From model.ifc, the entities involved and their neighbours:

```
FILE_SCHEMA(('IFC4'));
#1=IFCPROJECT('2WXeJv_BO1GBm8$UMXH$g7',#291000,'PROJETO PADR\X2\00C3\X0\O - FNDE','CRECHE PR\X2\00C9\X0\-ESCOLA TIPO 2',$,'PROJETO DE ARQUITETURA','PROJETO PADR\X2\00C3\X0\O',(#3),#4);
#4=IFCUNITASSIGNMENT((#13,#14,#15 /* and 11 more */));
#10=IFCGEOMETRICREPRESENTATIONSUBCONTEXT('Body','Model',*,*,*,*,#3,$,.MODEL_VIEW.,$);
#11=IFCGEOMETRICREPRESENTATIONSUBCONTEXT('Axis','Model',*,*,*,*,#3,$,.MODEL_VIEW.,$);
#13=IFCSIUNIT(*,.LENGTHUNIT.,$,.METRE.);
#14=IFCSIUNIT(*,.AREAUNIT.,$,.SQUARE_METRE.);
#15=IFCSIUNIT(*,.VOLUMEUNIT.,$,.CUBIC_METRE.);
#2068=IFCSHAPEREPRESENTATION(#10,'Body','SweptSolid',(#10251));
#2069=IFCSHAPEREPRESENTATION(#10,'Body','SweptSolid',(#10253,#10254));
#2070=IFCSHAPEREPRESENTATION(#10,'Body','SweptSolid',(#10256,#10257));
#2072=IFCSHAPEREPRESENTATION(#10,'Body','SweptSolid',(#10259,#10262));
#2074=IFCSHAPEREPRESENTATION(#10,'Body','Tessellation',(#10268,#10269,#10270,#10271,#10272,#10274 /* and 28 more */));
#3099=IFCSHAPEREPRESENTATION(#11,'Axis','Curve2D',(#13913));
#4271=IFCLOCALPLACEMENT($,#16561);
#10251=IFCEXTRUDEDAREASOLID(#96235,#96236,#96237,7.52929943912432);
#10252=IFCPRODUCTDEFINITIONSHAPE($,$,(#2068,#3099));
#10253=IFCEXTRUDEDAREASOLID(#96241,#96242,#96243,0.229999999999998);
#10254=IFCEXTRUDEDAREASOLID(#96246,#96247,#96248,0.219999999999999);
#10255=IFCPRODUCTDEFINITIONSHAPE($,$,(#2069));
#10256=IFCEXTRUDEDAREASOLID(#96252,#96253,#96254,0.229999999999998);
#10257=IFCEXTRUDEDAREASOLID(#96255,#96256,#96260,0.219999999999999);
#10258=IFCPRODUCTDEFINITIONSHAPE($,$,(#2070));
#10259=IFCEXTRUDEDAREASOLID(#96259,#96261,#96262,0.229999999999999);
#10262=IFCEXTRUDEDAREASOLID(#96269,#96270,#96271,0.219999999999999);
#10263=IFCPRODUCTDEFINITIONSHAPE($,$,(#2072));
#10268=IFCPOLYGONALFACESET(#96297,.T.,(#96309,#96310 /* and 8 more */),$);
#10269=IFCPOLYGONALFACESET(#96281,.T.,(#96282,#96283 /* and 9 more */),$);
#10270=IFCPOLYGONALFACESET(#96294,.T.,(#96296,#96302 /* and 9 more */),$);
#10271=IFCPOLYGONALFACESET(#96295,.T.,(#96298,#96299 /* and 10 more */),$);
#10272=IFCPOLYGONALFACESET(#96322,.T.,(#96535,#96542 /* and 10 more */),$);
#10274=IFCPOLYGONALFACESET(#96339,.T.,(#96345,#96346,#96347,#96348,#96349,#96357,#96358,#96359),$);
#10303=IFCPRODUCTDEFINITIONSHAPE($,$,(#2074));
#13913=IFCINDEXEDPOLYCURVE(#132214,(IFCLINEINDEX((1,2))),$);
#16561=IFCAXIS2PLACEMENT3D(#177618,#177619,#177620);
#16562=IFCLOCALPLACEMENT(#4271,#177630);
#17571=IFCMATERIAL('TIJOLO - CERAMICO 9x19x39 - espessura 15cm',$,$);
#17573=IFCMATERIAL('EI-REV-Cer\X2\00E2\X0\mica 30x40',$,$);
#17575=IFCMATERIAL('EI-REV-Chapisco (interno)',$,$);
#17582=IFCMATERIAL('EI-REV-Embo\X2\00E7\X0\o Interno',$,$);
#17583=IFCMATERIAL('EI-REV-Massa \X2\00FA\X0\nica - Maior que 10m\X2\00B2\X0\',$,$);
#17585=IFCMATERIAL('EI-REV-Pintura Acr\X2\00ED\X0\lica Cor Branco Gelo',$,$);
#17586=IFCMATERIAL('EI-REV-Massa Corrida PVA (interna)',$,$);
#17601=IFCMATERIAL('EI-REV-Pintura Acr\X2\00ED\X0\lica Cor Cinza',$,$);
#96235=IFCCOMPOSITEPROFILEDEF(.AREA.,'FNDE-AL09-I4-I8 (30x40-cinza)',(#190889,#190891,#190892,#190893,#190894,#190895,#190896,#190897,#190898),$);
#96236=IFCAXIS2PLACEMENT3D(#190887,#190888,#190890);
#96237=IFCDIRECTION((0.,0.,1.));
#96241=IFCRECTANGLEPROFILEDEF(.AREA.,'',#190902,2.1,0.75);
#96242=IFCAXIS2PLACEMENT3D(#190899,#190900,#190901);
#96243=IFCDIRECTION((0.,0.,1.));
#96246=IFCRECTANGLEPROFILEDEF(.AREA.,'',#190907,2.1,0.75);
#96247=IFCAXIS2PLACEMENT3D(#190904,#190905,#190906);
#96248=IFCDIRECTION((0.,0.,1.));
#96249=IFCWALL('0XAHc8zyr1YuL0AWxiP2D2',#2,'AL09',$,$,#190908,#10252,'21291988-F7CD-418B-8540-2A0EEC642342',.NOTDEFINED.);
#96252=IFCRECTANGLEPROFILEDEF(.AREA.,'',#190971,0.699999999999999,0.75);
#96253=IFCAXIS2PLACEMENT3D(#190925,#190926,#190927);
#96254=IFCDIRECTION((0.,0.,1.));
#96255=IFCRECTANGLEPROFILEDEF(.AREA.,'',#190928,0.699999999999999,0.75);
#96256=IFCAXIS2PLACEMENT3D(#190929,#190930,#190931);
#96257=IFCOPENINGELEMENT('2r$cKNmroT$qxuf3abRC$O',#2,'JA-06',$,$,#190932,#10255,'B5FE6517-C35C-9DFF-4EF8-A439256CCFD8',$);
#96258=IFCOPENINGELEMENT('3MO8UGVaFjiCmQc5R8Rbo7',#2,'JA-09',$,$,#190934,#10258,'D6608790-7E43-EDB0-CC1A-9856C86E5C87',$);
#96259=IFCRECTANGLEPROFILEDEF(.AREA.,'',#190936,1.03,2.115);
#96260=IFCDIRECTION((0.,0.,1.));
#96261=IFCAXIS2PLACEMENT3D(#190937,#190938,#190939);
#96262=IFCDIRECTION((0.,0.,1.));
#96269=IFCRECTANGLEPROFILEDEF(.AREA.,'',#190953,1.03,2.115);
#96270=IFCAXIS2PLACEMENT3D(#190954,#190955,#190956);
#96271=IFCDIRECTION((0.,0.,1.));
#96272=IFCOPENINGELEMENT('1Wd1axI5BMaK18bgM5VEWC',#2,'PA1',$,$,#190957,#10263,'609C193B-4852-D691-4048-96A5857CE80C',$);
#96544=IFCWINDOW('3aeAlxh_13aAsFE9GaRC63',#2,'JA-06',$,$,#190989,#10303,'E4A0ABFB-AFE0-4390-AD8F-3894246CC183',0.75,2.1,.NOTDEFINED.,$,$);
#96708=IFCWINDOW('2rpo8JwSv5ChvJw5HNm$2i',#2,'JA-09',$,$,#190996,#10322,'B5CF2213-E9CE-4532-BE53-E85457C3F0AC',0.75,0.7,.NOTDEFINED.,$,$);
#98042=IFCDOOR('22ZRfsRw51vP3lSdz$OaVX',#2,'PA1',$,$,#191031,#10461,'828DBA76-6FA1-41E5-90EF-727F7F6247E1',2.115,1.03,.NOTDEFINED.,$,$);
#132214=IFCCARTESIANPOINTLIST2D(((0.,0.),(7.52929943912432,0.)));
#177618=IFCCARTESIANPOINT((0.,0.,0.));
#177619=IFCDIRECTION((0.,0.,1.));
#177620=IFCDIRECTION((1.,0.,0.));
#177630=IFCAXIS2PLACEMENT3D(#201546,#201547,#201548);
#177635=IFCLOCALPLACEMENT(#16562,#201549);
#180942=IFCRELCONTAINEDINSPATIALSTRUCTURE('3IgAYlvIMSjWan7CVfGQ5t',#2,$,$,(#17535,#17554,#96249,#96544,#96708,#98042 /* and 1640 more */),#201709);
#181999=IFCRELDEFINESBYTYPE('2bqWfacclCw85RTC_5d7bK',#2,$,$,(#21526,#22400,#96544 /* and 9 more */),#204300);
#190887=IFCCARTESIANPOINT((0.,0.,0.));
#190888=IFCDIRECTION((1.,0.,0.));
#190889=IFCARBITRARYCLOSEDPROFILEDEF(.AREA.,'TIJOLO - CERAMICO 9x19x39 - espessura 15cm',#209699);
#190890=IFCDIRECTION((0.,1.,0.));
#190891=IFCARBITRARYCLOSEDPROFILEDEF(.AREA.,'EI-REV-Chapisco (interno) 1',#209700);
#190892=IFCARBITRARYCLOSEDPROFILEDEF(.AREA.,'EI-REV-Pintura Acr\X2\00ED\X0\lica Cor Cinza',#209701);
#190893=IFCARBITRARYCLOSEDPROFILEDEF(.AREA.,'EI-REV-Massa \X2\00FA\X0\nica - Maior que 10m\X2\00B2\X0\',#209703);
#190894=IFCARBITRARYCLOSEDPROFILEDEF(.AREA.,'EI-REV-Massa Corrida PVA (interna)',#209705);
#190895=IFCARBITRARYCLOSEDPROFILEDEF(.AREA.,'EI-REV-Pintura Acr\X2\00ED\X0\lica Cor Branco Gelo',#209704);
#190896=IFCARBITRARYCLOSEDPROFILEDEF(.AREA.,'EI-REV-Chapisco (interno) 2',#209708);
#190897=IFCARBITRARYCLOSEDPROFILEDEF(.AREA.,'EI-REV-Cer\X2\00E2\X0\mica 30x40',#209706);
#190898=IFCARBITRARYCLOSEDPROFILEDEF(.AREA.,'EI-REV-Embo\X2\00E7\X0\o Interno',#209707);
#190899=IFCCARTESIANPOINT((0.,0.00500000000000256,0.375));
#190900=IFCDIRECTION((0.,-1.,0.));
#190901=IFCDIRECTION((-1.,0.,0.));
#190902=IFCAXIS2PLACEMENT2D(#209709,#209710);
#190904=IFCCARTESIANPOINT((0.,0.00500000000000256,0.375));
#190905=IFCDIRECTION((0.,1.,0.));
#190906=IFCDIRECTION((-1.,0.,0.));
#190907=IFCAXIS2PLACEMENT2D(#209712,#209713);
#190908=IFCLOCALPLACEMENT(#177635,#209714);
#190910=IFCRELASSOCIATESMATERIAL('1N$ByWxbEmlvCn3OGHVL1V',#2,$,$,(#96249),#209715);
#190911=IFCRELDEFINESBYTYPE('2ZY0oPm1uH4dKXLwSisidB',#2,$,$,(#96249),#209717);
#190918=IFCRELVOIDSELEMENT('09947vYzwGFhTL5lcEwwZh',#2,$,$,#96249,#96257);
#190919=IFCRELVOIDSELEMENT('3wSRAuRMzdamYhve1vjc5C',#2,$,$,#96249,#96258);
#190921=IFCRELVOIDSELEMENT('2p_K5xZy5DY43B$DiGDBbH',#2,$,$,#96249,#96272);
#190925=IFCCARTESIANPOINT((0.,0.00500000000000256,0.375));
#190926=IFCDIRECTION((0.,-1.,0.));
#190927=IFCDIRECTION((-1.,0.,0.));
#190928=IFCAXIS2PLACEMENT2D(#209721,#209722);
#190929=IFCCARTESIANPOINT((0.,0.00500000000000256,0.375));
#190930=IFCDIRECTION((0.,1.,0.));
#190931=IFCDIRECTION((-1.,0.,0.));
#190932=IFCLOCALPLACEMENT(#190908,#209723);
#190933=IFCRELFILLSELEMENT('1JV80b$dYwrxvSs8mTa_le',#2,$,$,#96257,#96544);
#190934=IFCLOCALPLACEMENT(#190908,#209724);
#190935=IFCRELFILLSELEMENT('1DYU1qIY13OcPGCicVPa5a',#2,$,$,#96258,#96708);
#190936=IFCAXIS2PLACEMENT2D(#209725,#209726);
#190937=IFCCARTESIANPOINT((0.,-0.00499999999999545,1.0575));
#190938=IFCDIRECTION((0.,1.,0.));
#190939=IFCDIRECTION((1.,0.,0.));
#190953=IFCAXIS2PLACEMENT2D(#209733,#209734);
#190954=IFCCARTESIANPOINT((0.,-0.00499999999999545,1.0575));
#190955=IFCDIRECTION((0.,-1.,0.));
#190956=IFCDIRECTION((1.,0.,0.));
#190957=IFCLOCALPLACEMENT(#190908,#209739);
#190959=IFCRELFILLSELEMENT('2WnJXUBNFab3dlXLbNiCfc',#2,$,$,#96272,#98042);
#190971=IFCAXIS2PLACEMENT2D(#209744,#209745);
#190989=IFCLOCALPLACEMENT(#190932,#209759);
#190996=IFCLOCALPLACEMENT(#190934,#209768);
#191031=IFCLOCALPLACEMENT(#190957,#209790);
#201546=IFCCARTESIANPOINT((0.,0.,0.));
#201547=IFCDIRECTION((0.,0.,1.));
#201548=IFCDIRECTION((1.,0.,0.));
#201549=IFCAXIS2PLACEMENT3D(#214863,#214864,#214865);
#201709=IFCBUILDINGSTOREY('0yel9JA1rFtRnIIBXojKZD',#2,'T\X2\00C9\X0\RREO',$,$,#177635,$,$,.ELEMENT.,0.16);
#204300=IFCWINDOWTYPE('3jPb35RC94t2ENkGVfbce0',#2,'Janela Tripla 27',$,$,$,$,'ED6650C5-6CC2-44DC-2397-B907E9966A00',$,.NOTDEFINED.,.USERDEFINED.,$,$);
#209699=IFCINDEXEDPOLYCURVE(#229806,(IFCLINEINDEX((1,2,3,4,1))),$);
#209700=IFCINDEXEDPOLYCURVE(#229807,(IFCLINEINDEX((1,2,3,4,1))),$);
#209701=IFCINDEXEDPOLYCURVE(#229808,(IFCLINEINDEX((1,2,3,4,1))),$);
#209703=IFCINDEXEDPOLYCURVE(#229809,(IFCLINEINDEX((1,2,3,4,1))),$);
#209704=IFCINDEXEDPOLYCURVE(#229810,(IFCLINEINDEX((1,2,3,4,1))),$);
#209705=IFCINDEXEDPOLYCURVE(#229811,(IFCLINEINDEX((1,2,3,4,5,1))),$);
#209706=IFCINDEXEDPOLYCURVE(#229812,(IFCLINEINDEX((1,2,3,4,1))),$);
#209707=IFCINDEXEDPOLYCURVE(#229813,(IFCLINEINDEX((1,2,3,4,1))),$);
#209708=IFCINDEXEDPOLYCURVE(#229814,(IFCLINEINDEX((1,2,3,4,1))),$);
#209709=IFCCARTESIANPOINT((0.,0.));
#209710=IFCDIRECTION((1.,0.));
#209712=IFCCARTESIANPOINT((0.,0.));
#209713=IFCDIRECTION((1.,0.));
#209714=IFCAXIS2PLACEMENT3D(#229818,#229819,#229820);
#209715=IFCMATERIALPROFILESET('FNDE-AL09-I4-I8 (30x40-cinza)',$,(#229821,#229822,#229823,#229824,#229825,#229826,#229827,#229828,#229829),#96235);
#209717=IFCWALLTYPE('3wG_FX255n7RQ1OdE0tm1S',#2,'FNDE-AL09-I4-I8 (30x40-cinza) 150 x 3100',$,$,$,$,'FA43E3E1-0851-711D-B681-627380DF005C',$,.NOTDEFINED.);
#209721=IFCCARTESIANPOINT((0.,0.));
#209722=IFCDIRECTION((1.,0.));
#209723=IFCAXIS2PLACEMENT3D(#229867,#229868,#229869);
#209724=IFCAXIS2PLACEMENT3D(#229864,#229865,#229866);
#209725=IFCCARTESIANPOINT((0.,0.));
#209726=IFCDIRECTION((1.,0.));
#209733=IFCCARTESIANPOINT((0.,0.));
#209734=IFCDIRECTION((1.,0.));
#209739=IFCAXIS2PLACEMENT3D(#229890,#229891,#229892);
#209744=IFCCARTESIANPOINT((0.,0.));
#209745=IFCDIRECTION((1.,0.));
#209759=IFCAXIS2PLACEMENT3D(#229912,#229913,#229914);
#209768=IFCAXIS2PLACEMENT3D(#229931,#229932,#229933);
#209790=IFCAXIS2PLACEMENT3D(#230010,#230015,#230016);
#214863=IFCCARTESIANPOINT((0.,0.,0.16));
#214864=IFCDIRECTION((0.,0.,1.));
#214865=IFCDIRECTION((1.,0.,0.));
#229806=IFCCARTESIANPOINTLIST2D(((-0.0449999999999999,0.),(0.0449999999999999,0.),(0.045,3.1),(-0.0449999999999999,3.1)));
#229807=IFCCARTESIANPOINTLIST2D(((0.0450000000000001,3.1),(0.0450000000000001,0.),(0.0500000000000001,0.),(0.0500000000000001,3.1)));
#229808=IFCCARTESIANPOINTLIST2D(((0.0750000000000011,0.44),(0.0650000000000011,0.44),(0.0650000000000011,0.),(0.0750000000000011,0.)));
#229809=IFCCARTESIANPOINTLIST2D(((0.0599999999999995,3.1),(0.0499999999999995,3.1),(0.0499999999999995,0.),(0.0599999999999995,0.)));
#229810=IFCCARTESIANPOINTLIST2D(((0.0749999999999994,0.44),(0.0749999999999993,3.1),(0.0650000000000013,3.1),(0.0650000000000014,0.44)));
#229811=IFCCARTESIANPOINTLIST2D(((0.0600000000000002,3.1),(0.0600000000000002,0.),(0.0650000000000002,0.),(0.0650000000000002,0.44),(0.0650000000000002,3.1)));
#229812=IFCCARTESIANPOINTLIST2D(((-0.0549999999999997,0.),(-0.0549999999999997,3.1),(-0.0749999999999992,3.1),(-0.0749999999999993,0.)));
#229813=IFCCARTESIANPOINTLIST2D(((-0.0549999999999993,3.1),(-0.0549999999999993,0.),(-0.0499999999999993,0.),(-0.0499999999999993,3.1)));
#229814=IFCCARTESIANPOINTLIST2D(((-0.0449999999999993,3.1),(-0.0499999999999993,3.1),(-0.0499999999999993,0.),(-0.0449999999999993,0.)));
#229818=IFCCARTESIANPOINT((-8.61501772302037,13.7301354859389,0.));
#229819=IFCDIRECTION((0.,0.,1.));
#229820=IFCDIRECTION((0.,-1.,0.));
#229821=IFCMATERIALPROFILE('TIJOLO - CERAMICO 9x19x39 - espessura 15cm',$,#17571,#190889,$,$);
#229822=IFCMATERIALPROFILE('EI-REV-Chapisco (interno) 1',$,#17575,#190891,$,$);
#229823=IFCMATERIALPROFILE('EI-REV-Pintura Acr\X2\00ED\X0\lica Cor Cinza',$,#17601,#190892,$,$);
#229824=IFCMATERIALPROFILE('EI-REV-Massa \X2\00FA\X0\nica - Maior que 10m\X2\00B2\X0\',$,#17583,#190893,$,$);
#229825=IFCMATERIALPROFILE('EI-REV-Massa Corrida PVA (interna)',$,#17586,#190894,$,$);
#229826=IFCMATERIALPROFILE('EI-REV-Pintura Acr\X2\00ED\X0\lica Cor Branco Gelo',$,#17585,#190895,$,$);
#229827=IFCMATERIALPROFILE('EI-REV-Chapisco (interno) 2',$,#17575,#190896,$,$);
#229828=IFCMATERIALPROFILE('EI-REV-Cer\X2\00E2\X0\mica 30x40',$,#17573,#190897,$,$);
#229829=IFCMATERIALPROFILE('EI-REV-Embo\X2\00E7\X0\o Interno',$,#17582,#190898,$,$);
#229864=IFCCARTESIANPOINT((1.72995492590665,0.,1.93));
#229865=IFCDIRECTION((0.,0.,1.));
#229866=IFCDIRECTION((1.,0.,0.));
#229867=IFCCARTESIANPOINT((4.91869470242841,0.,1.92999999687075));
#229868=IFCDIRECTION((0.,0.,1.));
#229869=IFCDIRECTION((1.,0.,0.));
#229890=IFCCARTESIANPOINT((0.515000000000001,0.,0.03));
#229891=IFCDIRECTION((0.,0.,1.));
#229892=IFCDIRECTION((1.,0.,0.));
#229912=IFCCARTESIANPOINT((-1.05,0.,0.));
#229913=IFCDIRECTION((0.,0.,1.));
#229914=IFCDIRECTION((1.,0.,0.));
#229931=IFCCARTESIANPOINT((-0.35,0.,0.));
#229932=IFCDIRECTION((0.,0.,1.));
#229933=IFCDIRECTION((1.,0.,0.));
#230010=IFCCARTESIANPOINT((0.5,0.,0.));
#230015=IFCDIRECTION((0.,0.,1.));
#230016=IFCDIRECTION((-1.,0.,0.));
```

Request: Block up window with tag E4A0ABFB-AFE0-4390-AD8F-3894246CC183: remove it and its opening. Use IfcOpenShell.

```python
import ifcopenshell
import ifcopenshell.api.feature
import ifcopenshell.api.root
import ifcopenshell.geom
import ifcopenshell.util.shape

model = ifcopenshell.open("model.ifc")
settings = ifcopenshell.geom.settings()


def volume(element):
    """Net volume in cubic metres, openings subtracted."""
    shape = ifcopenshell.geom.create_shape(settings, element)
    return ifcopenshell.util.shape.get_volume(shape.geometry)


window = model.by_guid("3aeAlxh_13aAsFE9GaRC63")
opening = window.FillsVoids[0].RelatingOpeningElement
wall = opening.VoidsElements[0].RelatingBuildingElement
before = volume(wall)

ifcopenshell.api.root.remove_product(model, product=window)
ifcopenshell.api.feature.remove_feature(model, feature=opening)

after = volume(wall)

print(f"wall volume {before:.3f} -> {after:.3f} m3")

model.write("model_v2.ifc")
```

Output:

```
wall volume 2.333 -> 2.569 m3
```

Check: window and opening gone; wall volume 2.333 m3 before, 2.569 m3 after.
